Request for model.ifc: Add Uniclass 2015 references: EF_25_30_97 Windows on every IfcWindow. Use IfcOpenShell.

First a look at what the model holds.

```python
import ifcopenshell

model = ifcopenshell.open("model.ifc")
print(model.schema)
print("classifications:", [c.Name for c in model.by_type("IfcClassification")])
for ifc_class in ("IfcDoor", "IfcRoof", "IfcStair", "IfcWall", "IfcWindow"):
    print(ifc_class, len(model.by_type(ifc_class)))
```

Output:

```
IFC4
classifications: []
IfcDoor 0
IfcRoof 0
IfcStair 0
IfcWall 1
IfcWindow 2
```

```python
import ifcopenshell
import ifcopenshell.api.classification

model = ifcopenshell.open("model.ifc")

system = ifcopenshell.api.classification.add_classification(model, classification="Uniclass 2015")

codes = {
    "IfcWindow": ("EF_25_30_97", "Windows"),
}
for ifc_class, (code, name) in codes.items():
    products = model.by_type(ifc_class)
    ifcopenshell.api.classification.add_reference(
        model, products=products, classification=system, identification=code, name=name
    )
    print(code, len(products))

model.write("model_updated.ifc")
```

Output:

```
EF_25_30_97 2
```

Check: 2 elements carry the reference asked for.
